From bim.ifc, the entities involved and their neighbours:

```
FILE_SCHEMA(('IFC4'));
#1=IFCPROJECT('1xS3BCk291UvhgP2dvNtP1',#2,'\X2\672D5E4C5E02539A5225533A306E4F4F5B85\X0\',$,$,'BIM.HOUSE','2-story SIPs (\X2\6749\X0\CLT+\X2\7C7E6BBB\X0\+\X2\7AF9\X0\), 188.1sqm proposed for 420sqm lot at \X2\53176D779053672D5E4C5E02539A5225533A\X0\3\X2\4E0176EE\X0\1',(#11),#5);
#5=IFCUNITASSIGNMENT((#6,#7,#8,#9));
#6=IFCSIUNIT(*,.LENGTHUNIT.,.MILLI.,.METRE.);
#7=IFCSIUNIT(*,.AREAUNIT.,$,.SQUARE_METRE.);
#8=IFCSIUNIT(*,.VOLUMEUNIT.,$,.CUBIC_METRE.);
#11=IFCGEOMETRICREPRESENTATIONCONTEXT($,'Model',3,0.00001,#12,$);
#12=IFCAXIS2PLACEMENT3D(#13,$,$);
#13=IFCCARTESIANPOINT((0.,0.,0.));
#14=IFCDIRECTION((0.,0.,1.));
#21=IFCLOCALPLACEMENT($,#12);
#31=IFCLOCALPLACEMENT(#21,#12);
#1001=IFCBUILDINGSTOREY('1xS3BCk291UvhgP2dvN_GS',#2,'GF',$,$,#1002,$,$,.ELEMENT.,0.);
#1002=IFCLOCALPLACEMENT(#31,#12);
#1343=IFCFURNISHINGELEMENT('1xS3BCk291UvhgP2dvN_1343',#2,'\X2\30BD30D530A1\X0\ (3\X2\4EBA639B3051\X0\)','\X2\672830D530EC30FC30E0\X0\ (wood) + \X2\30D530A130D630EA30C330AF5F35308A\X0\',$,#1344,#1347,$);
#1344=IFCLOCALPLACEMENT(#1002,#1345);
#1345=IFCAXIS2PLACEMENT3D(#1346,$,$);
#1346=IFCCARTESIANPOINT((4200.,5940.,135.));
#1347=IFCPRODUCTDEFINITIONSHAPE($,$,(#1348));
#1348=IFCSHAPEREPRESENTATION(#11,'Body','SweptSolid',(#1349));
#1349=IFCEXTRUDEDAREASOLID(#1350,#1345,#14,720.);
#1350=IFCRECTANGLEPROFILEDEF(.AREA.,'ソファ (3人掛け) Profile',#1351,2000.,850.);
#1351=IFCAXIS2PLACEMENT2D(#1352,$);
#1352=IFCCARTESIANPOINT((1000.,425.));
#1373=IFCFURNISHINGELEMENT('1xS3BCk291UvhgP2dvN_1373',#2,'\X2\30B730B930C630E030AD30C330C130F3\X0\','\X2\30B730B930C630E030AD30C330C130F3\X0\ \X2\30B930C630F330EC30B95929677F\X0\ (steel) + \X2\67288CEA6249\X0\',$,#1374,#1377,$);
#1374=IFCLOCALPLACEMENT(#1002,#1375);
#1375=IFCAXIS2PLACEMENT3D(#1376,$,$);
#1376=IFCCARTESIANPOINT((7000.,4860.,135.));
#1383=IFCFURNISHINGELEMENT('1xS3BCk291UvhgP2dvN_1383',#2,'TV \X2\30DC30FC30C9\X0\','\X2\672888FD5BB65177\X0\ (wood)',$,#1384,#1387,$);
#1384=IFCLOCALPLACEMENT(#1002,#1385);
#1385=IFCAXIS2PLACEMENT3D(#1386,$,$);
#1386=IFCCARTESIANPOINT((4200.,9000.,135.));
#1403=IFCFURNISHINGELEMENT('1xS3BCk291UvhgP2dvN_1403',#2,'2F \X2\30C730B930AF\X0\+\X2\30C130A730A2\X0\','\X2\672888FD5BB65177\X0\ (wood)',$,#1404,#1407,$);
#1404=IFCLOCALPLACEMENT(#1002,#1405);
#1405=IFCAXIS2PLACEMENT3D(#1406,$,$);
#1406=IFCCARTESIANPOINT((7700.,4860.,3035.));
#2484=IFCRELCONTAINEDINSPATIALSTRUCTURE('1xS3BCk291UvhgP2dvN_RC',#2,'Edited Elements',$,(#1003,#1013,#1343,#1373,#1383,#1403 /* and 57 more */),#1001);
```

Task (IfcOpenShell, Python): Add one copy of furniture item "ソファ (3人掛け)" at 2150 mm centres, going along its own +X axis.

```python
import ifcopenshell
import ifcopenshell.api.geometry
import ifcopenshell.api.root
import ifcopenshell.util.element
import ifcopenshell.util.placement

model = ifcopenshell.open("bim.ifc")


def reuse_history(source, copy):
    """copy_class also copies each property set's owner history, people and application; keep the originals."""
    for rel in copy.IsDefinedBy:
        if rel.is_a("IfcRelDefinesByProperties") and (history := rel.RelatingPropertyDefinition.OwnerHistory):
            rel.RelatingPropertyDefinition.OwnerHistory = source.OwnerHistory
            ifcopenshell.util.element.remove_deep2(model, history)


source = model.by_guid("1xS3BCk291UvhgP2dvN_1343")
base = ifcopenshell.util.placement.get_local_placement(source.ObjectPlacement)
step = base[:3, 0] * 2150.0

for i in range(1, 2):
    copy = ifcopenshell.api.root.copy_class(model, product=source)
    copy.Representation = ifcopenshell.util.element.copy_deep(
        model, source.Representation, exclude=["IfcGeometricRepresentationContext", "IfcRepresentationMap"]
    )
    reuse_history(source, copy)
    matrix = base.copy()
    matrix[:3, 3] += i * step
    print("added at", matrix[:3, 3].round(3) + 0.0)
    ifcopenshell.api.geometry.edit_object_placement(model, product=copy, matrix=matrix, is_si=False)

model.write("bim_v2.ifc")
```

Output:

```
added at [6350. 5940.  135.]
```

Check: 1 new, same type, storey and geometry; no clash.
